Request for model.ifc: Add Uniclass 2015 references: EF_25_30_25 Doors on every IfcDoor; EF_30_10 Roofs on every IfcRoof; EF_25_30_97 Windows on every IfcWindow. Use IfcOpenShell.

First a look at what the model holds.

```python
import ifcopenshell

model = ifcopenshell.open("model.ifc")
print(model.schema)
print("classifications:", [c.Name for c in model.by_type("IfcClassification")])
for ifc_class in ("IfcDoor", "IfcRoof", "IfcStair", "IfcWall", "IfcWindow"):
    print(ifc_class, len(model.by_type(ifc_class)))
```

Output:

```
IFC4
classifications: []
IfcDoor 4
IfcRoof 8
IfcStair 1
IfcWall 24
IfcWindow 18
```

```python
import ifcopenshell
import ifcopenshell.api.classification

model = ifcopenshell.open("model.ifc")

system = ifcopenshell.api.classification.add_classification(model, classification="Uniclass 2015")

codes = {
    "IfcDoor": ("EF_25_30_25", "Doors"),
    "IfcRoof": ("EF_30_10", "Roofs"),
    "IfcWindow": ("EF_25_30_97", "Windows"),
}
for ifc_class, (code, name) in codes.items():
    products = model.by_type(ifc_class)
    ifcopenshell.api.classification.add_reference(
        model, products=products, classification=system, identification=code, name=name
    )
    print(code, len(products))

model.write("model_rev.ifc")
```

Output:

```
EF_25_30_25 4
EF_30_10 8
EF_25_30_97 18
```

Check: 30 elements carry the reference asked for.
